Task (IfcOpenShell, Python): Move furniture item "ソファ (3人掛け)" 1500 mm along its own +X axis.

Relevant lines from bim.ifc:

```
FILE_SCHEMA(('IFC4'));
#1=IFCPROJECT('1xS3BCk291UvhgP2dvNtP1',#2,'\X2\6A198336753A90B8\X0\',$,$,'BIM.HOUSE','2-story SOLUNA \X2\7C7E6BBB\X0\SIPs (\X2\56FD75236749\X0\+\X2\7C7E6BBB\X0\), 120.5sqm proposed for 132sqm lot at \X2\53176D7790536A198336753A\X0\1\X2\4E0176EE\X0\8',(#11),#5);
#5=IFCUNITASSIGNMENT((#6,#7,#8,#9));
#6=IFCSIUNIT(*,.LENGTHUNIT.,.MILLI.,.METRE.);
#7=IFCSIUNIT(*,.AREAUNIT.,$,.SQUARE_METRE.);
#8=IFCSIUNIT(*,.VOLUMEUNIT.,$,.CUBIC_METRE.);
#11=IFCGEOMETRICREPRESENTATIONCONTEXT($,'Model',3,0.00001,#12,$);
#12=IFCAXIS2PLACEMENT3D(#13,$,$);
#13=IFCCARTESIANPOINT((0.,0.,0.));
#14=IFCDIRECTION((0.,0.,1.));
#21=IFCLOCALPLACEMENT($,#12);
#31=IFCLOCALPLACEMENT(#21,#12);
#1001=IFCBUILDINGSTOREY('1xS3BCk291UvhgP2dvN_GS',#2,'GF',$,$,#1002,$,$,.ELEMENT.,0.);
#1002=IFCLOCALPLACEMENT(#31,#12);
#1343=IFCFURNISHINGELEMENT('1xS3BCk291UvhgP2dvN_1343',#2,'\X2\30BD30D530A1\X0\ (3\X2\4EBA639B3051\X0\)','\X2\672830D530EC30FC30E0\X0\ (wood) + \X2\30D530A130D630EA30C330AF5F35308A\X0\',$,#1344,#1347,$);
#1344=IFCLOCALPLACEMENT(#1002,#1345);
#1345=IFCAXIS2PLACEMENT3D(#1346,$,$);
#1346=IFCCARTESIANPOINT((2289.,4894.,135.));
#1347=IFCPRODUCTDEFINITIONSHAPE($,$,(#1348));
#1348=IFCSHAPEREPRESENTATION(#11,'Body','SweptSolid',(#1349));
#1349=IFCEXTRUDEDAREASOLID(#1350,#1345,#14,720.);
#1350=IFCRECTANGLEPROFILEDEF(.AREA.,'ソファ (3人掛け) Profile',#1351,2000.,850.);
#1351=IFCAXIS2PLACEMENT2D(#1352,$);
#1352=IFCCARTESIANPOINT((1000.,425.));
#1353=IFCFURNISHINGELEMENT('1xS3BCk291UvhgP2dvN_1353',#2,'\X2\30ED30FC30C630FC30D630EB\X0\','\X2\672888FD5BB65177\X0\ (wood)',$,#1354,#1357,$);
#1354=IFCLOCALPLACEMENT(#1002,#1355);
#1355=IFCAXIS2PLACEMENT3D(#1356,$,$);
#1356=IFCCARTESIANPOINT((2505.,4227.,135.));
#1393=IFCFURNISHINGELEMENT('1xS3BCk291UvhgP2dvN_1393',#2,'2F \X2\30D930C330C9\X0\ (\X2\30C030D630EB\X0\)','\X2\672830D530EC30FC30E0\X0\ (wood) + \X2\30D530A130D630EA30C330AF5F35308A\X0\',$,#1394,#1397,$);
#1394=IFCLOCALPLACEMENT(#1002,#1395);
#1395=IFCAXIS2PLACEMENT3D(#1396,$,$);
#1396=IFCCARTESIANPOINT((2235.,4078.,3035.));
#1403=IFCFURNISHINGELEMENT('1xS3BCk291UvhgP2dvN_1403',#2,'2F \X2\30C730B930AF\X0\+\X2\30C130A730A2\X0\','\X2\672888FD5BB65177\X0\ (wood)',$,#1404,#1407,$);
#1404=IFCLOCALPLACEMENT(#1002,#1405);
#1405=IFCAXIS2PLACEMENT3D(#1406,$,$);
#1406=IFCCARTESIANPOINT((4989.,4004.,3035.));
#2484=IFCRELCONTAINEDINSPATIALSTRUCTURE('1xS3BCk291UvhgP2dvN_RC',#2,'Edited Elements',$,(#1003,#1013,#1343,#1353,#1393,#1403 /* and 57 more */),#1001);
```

```python
import ifcopenshell
import ifcopenshell.api.geometry
import ifcopenshell.util.placement
import ifcopenshell.util.unit

model = ifcopenshell.open("bim.ifc")
unit_scale = ifcopenshell.util.unit.calculate_unit_scale(model)

item = model.by_id(1343)
matrix = ifcopenshell.util.placement.get_local_placement(item.ObjectPlacement)
matrix[:3, 3] += matrix[:3, 0] * 1.5 / unit_scale
ifcopenshell.api.geometry.edit_object_placement(model, product=item, matrix=matrix, is_si=False)

print(ifcopenshell.util.placement.get_local_placement(item.ObjectPlacement).round(3) + 0.0)

model.write("bim_v2.ifc")
```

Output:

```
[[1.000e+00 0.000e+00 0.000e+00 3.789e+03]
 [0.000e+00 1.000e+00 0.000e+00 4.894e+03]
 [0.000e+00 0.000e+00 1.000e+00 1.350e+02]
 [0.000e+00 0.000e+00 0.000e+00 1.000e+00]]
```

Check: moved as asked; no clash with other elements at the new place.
